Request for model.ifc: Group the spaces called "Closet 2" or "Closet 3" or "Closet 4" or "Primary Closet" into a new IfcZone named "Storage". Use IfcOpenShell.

First a look at what the model holds.

```python
import ifcopenshell

model = ifcopenshell.open("model.ifc")
print(model.schema)
seen = {}
for space in model.by_type("IfcSpace"):
    seen[space.LongName] = seen.get(space.LongName, 0) + 1
for name, count in sorted(seen.items(), key=str):
    print(count, "x", name)
print("zones:", [z.Name for z in model.by_type("IfcZone")][:20])
```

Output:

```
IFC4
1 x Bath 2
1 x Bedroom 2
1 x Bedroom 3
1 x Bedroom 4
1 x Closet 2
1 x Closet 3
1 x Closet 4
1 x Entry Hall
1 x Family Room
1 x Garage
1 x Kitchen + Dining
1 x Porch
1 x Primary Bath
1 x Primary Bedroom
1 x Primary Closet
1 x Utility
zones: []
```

```python
import ifcopenshell
import ifcopenshell.api.group
import ifcopenshell.api.root

model = ifcopenshell.open("model.ifc")

names = {"Closet 2", "Closet 3", "Closet 4", "Primary Closet"}
spaces = [s for s in model.by_type("IfcSpace") if s.LongName in names]

zone = ifcopenshell.api.root.create_entity(model, ifc_class="IfcZone", name="Storage")
ifcopenshell.api.group.assign_group(model, products=spaces, group=zone)
print(len(spaces), "spaces in", zone.Name)

model.write("model_updated.ifc")
```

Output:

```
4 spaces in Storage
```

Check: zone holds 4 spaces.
